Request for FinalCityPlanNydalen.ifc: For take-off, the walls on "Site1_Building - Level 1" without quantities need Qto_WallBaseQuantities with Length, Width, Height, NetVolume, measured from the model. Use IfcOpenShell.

First a look at what the model holds.

```python
import ifcopenshell
import ifcopenshell.util.element
import ifcopenshell.util.unit

model = ifcopenshell.open("FinalCityPlanNydalen.ifc")
print(model.schema)
for unit_type in ("LENGTHUNIT", "AREAUNIT", "VOLUMEUNIT"):
    print(unit_type, ifcopenshell.util.unit.calculate_unit_scale(model, unit_type))
storey = next(s for s in model.by_type("IfcBuildingStorey") if s.Name == "Site1_Building - Level 1")
walls = [e for e in ifcopenshell.util.element.get_decomposition(storey) if e.is_a("IfcWall")]
for e in sorted(walls, key=lambda e: e.id()):
    print(e.id(), e.is_a(), e.Name, list(ifcopenshell.util.element.get_psets(e, qtos_only=True)), sep=" | ")
```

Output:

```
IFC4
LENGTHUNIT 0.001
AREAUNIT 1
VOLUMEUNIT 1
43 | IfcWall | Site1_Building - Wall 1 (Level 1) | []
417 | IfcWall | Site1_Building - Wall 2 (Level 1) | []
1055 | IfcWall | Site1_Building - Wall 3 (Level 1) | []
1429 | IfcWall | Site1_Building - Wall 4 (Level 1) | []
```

```python
import ifcopenshell
import ifcopenshell.api.pset
import ifcopenshell.geom
import ifcopenshell.util.element
import ifcopenshell.util.shape
import ifcopenshell.util.unit

model = ifcopenshell.open("FinalCityPlanNydalen.ifc")
unit_scale = ifcopenshell.util.unit.calculate_unit_scale(model)
volume_scale = ifcopenshell.util.unit.calculate_unit_scale(model, "VOLUMEUNIT")
settings = ifcopenshell.geom.settings()

storey = next(s for s in model.by_type("IfcBuildingStorey") if s.Name == "Site1_Building - Level 1")
walls = [e for e in ifcopenshell.util.element.get_decomposition(storey) if e.is_a("IfcWall")]

for e in sorted(walls, key=lambda e: e.id()):
    if ifcopenshell.util.element.get_psets(e, qtos_only=True, should_inherit=False):
        continue
    # Geometry comes back in metres, in the element's own axes.
    shape = ifcopenshell.geom.create_shape(settings, e)
    values = {
        "Length": ifcopenshell.util.shape.get_x(shape.geometry) / unit_scale,
        "Width": ifcopenshell.util.shape.get_y(shape.geometry) / unit_scale,
        "Height": ifcopenshell.util.shape.get_z(shape.geometry) / unit_scale,
        "NetVolume": ifcopenshell.util.shape.get_volume(shape.geometry) / volume_scale,
    }
    qto = ifcopenshell.api.pset.add_qto(model, product=e, name="Qto_WallBaseQuantities")
    ifcopenshell.api.pset.edit_qto(model, qto=qto, properties=values)
    print(e.id(), {k: round(v, 3) for k, v in values.items()})

model.write("FinalCityPlanNydalen_rev.ifc")
```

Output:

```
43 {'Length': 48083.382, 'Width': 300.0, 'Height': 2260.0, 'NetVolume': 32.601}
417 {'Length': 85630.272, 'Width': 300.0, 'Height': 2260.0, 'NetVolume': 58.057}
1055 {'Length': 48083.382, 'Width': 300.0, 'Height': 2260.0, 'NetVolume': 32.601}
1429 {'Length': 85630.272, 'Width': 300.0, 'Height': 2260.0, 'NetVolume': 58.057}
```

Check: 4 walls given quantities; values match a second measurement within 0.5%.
